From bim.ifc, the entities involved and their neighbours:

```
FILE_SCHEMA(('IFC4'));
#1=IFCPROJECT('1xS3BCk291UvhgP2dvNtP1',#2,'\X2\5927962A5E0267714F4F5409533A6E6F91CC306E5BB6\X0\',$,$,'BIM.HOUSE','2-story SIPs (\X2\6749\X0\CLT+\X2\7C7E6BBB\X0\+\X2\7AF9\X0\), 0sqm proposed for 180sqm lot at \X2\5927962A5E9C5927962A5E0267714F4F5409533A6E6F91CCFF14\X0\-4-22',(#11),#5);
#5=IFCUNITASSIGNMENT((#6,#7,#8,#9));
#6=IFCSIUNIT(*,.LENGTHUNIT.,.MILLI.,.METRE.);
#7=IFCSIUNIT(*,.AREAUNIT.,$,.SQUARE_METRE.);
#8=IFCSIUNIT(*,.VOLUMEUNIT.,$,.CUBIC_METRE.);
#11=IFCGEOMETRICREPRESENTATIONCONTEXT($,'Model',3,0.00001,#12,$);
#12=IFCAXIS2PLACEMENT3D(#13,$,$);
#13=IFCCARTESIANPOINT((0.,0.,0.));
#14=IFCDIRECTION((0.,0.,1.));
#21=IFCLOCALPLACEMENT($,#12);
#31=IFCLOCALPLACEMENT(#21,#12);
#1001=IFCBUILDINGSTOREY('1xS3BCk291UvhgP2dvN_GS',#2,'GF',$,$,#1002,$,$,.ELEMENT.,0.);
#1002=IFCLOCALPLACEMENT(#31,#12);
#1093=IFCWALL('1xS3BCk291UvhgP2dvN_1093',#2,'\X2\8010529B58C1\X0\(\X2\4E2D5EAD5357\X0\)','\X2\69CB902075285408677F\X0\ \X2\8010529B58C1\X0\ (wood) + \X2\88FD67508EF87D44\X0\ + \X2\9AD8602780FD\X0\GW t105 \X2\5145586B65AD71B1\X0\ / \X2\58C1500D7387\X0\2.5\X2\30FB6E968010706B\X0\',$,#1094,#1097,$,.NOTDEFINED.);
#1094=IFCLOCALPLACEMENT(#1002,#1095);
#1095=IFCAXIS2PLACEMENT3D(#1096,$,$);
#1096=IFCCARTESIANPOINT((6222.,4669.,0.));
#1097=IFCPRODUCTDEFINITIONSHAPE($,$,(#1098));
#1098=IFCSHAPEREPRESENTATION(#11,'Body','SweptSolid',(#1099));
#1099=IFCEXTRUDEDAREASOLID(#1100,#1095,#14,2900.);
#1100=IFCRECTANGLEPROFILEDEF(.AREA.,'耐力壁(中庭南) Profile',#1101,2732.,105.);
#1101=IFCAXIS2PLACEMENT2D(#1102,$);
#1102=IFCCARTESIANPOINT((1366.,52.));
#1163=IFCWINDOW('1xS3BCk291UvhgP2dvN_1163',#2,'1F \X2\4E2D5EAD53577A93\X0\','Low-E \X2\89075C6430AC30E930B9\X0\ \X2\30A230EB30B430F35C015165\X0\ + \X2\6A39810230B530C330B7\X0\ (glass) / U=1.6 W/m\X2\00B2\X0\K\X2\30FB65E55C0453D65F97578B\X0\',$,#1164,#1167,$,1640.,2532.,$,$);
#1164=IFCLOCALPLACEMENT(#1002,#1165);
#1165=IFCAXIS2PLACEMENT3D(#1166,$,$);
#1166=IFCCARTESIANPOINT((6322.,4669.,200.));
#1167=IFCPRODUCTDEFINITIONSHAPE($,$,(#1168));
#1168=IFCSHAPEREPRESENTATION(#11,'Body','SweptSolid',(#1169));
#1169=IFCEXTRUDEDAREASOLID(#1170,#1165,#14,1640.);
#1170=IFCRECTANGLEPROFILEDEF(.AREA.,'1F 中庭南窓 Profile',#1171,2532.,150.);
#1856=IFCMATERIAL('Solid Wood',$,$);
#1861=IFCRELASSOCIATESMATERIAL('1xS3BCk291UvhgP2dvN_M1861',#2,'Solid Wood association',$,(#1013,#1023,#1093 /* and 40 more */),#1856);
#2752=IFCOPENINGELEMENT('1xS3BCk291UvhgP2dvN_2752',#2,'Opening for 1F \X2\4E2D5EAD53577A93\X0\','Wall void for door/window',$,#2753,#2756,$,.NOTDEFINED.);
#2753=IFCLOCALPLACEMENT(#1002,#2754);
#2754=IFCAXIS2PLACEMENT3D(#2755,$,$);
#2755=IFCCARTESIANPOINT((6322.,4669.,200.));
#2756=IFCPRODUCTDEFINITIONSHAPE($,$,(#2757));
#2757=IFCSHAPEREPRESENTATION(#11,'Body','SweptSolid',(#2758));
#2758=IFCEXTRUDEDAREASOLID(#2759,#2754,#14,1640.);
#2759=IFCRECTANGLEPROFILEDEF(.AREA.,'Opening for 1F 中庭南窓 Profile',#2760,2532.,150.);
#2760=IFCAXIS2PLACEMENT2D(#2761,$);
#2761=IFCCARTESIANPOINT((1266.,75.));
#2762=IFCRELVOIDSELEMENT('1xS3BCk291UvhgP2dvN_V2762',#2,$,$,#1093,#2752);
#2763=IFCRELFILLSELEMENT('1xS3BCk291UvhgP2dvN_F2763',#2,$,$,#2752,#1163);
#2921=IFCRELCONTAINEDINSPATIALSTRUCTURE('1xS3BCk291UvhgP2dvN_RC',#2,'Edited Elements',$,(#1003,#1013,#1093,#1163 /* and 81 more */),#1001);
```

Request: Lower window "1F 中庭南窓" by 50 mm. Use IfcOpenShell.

```python
import numpy as np
import ifcopenshell
import ifcopenshell.api.geometry
import ifcopenshell.util.placement
import ifcopenshell.util.unit

model = ifcopenshell.open("bim.ifc")
unit_scale = ifcopenshell.util.unit.calculate_unit_scale(model)

window = model.by_guid("1xS3BCk291UvhgP2dvN_1163")
opening = window.FillsVoids[0].RelatingOpeningElement
dz = -50.0

shift = np.array([0.0, 0.0, dz])
# The window is not placed relative to its opening, so move both.
for product in (opening, window):
    matrix = ifcopenshell.util.placement.get_local_placement(product.ObjectPlacement)
    matrix[:3, 3] += shift
    ifcopenshell.api.geometry.edit_object_placement(model, product=product, matrix=matrix, is_si=False)

print(f"moved by {dz * unit_scale:+.3f} m")

model.write("bim-out.ifc")
```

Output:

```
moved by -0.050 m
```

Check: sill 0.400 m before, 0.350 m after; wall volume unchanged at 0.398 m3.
